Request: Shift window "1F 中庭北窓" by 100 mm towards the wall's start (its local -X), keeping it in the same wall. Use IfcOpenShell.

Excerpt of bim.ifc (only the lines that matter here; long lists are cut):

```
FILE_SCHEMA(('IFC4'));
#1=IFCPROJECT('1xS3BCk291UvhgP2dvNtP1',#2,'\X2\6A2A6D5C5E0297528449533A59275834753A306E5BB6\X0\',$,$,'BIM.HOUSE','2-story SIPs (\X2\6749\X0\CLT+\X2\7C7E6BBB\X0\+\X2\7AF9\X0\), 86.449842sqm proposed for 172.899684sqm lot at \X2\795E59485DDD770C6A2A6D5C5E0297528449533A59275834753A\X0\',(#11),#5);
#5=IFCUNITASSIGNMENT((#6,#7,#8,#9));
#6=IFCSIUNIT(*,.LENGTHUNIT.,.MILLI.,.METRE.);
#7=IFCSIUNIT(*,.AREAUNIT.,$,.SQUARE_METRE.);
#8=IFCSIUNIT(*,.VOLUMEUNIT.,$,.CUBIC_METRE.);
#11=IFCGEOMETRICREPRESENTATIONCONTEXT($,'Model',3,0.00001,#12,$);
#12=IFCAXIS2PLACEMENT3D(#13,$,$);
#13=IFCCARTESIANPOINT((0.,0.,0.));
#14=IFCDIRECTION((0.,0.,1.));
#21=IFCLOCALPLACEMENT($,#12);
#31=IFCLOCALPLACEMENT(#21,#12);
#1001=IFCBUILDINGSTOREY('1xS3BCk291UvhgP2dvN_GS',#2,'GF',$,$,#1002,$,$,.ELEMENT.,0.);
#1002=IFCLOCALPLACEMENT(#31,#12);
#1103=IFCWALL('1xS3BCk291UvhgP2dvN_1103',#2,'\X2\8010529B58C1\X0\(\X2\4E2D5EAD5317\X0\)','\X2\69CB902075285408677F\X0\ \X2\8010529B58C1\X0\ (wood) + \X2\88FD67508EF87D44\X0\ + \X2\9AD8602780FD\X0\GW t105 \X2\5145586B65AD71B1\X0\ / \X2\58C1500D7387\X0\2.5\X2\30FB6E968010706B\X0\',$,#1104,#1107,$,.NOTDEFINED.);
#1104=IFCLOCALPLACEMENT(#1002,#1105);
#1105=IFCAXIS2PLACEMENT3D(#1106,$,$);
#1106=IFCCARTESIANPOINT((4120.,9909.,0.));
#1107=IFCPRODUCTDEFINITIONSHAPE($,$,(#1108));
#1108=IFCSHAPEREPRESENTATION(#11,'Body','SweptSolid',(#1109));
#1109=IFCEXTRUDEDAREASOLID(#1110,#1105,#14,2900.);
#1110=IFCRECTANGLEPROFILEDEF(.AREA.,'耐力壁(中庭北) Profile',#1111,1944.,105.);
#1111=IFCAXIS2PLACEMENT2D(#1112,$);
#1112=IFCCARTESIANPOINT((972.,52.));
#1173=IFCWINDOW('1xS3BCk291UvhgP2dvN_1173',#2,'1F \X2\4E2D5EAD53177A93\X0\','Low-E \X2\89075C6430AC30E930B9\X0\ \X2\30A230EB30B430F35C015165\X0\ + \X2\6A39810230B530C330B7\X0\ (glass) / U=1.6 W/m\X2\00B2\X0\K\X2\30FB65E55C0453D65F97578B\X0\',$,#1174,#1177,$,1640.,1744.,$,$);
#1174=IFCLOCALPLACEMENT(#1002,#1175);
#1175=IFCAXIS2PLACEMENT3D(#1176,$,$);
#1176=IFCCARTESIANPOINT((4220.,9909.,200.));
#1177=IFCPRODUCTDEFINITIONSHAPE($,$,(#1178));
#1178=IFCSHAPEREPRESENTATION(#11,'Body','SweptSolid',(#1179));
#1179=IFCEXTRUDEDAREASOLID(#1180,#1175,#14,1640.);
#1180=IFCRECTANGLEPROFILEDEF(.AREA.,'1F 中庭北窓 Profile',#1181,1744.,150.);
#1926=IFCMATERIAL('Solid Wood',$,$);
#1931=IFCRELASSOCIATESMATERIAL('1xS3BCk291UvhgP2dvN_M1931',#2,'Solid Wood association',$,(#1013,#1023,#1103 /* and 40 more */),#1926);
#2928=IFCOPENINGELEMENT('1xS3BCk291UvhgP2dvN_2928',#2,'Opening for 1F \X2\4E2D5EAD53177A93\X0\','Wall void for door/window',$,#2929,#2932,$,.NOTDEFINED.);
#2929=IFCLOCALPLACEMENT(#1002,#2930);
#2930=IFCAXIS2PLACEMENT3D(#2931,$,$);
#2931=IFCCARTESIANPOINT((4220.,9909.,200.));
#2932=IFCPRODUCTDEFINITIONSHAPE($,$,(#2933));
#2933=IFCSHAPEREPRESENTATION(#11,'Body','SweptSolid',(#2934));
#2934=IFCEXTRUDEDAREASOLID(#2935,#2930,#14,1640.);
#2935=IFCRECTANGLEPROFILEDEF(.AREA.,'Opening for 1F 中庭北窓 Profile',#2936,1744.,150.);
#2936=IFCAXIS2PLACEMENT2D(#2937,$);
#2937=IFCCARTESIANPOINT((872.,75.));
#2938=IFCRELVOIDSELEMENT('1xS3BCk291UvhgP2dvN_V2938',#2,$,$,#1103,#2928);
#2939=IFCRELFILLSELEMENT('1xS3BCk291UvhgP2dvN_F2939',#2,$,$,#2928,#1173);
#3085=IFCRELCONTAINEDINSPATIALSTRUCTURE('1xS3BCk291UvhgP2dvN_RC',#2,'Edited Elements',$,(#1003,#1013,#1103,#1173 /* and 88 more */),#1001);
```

```python
import ifcopenshell
import ifcopenshell.api.geometry
import ifcopenshell.util.placement
import ifcopenshell.util.unit

model = ifcopenshell.open("bim.ifc")
unit_scale = ifcopenshell.util.unit.calculate_unit_scale(model)

window = model.by_guid("1xS3BCk291UvhgP2dvN_1173")
opening = window.FillsVoids[0].RelatingOpeningElement
wall = opening.VoidsElements[0].RelatingBuildingElement

wall_matrix = ifcopenshell.util.placement.get_local_placement(wall.ObjectPlacement)
shift = wall_matrix[:3, 0] * -0.1 / unit_scale
before = ifcopenshell.util.placement.get_local_placement(window.ObjectPlacement)[:3, 3].copy()

# The window is not placed relative to its opening, so move both.
for product in (opening, window):
    matrix = ifcopenshell.util.placement.get_local_placement(product.ObjectPlacement)
    matrix[:3, 3] += shift
    ifcopenshell.api.geometry.edit_object_placement(model, product=product, matrix=matrix, is_si=False)

after = ifcopenshell.util.placement.get_local_placement(window.ObjectPlacement)[:3, 3]
print("window moved by", (after - before).round(3) + 0.0)

model.write("bim_v2.ifc")
```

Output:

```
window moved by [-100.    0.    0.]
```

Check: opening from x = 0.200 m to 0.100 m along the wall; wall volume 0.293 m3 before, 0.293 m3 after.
